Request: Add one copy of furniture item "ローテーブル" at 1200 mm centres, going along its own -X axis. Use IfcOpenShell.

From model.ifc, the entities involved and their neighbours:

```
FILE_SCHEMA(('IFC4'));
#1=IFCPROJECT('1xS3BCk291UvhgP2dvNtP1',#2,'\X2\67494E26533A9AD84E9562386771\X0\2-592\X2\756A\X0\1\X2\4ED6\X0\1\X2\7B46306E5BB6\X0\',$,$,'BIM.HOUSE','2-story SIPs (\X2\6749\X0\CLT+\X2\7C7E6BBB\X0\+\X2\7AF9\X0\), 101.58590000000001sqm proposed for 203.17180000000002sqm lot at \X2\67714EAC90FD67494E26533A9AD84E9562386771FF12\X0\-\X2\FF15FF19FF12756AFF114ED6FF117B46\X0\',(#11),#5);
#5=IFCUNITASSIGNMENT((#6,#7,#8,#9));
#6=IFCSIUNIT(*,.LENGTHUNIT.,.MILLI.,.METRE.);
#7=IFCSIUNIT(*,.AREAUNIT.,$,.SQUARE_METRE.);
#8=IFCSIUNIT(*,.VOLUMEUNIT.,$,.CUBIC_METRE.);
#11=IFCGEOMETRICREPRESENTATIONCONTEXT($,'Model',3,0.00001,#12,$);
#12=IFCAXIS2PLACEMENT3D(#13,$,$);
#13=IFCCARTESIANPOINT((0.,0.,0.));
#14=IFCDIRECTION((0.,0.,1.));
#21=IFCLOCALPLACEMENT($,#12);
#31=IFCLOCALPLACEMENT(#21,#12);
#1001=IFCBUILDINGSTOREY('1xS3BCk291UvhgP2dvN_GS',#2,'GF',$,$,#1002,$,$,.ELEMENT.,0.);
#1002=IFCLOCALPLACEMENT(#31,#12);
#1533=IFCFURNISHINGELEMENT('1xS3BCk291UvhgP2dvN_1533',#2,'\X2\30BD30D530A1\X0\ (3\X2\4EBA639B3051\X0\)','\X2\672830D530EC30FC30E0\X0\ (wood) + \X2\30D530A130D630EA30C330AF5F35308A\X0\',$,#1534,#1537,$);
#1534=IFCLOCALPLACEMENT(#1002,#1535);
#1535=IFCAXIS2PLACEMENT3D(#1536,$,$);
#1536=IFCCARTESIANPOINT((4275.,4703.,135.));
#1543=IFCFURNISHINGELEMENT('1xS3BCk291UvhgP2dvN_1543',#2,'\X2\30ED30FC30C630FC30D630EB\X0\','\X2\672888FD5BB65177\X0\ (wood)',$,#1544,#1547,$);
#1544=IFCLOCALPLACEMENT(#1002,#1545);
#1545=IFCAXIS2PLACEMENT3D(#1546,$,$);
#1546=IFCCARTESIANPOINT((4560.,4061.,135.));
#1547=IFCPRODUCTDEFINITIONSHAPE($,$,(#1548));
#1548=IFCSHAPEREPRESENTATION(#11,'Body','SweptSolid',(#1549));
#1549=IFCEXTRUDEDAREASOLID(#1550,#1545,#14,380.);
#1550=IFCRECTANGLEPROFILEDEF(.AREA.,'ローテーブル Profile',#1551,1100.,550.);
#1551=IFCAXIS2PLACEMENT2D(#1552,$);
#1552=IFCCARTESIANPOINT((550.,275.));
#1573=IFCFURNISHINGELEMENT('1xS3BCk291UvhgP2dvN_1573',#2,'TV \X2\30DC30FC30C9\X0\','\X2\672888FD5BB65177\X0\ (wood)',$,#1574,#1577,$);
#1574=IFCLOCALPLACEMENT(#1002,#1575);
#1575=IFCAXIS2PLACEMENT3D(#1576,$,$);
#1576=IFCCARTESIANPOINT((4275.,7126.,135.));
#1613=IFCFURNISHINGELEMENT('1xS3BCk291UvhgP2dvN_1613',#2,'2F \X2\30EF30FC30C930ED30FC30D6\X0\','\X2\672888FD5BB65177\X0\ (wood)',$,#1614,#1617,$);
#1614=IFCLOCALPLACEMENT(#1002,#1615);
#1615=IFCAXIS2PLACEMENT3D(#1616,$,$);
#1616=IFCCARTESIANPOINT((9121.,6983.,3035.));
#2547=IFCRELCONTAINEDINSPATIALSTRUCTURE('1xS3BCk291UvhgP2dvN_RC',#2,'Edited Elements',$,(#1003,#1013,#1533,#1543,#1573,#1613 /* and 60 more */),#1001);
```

```python
import ifcopenshell
import ifcopenshell.api.geometry
import ifcopenshell.api.root
import ifcopenshell.util.element
import ifcopenshell.util.placement
import ifcopenshell.util.unit

model = ifcopenshell.open("model.ifc")
unit_scale = ifcopenshell.util.unit.calculate_unit_scale(model)


def reuse_history(source, copy):
    """copy_class also copies each property set's owner history, people and application; keep the originals."""
    for rel in copy.IsDefinedBy:
        if rel.is_a("IfcRelDefinesByProperties") and (history := rel.RelatingPropertyDefinition.OwnerHistory):
            rel.RelatingPropertyDefinition.OwnerHistory = source.OwnerHistory
            ifcopenshell.util.element.remove_deep2(model, history)


source = model.by_guid("1xS3BCk291UvhgP2dvN_1543")
base = ifcopenshell.util.placement.get_local_placement(source.ObjectPlacement)
step = -base[:3, 0] * 1.2 / unit_scale

for i in range(1, 2):
    copy = ifcopenshell.api.root.copy_class(model, product=source)
    copy.Representation = ifcopenshell.util.element.copy_deep(
        model, source.Representation, exclude=["IfcGeometricRepresentationContext", "IfcRepresentationMap"]
    )
    reuse_history(source, copy)
    matrix = base.copy()
    matrix[:3, 3] += i * step
    print("added at", matrix[:3, 3].round(3) + 0.0)
    ifcopenshell.api.geometry.edit_object_placement(model, product=copy, matrix=matrix, is_si=False)

model.write("model_edited.ifc")
```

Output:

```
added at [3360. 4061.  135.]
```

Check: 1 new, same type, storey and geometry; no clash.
